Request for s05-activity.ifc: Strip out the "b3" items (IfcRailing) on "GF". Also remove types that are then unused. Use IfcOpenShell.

First a look at what the model holds.

```python
import ifcopenshell
import ifcopenshell.util.element

model = ifcopenshell.open("s05-activity.ifc")
print(model.schema)
storey = next(s for s in model.by_type("IfcBuildingStorey") if s.Name == "GF")
railings = [e for e in ifcopenshell.util.element.get_decomposition(storey) if e.is_a("IfcRailing")]
seen = {}
for e in railings:
    element_type = ifcopenshell.util.element.get_type(e)
    name = element_type.Name if element_type not in (None, e) else None
    seen[name] = seen.get(name, 0) + 1
for name, count in sorted(seen.items(), key=str):
    print(count, "x", name)
```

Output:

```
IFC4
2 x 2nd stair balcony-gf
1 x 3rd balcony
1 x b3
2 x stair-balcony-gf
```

```python
import ifcopenshell
import ifcopenshell.api.root
import ifcopenshell.util.element

model = ifcopenshell.open("s05-activity.ifc")

storey = next(s for s in model.by_type("IfcBuildingStorey") if s.Name == "GF")
railings = [e for e in ifcopenshell.util.element.get_decomposition(storey) if e.is_a("IfcRailing")]
targets = [e for e in railings if (t := ifcopenshell.util.element.get_type(e)) not in (None, e) and t.Name == "b3"]
types = {ifcopenshell.util.element.get_type(e) for e in targets} - {None, *targets}

for e in targets:
    ifcopenshell.api.root.remove_product(model, product=e)
print(len(targets), "removed")

unused = [t for t in types if not ifcopenshell.util.element.get_types(t)]
for t in unused:
    ifcopenshell.api.root.remove_product(model, product=t)
print(len(unused), "unused types removed")

model.write("s05-activity_updated.ifc")
```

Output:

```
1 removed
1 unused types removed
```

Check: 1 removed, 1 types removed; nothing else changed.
